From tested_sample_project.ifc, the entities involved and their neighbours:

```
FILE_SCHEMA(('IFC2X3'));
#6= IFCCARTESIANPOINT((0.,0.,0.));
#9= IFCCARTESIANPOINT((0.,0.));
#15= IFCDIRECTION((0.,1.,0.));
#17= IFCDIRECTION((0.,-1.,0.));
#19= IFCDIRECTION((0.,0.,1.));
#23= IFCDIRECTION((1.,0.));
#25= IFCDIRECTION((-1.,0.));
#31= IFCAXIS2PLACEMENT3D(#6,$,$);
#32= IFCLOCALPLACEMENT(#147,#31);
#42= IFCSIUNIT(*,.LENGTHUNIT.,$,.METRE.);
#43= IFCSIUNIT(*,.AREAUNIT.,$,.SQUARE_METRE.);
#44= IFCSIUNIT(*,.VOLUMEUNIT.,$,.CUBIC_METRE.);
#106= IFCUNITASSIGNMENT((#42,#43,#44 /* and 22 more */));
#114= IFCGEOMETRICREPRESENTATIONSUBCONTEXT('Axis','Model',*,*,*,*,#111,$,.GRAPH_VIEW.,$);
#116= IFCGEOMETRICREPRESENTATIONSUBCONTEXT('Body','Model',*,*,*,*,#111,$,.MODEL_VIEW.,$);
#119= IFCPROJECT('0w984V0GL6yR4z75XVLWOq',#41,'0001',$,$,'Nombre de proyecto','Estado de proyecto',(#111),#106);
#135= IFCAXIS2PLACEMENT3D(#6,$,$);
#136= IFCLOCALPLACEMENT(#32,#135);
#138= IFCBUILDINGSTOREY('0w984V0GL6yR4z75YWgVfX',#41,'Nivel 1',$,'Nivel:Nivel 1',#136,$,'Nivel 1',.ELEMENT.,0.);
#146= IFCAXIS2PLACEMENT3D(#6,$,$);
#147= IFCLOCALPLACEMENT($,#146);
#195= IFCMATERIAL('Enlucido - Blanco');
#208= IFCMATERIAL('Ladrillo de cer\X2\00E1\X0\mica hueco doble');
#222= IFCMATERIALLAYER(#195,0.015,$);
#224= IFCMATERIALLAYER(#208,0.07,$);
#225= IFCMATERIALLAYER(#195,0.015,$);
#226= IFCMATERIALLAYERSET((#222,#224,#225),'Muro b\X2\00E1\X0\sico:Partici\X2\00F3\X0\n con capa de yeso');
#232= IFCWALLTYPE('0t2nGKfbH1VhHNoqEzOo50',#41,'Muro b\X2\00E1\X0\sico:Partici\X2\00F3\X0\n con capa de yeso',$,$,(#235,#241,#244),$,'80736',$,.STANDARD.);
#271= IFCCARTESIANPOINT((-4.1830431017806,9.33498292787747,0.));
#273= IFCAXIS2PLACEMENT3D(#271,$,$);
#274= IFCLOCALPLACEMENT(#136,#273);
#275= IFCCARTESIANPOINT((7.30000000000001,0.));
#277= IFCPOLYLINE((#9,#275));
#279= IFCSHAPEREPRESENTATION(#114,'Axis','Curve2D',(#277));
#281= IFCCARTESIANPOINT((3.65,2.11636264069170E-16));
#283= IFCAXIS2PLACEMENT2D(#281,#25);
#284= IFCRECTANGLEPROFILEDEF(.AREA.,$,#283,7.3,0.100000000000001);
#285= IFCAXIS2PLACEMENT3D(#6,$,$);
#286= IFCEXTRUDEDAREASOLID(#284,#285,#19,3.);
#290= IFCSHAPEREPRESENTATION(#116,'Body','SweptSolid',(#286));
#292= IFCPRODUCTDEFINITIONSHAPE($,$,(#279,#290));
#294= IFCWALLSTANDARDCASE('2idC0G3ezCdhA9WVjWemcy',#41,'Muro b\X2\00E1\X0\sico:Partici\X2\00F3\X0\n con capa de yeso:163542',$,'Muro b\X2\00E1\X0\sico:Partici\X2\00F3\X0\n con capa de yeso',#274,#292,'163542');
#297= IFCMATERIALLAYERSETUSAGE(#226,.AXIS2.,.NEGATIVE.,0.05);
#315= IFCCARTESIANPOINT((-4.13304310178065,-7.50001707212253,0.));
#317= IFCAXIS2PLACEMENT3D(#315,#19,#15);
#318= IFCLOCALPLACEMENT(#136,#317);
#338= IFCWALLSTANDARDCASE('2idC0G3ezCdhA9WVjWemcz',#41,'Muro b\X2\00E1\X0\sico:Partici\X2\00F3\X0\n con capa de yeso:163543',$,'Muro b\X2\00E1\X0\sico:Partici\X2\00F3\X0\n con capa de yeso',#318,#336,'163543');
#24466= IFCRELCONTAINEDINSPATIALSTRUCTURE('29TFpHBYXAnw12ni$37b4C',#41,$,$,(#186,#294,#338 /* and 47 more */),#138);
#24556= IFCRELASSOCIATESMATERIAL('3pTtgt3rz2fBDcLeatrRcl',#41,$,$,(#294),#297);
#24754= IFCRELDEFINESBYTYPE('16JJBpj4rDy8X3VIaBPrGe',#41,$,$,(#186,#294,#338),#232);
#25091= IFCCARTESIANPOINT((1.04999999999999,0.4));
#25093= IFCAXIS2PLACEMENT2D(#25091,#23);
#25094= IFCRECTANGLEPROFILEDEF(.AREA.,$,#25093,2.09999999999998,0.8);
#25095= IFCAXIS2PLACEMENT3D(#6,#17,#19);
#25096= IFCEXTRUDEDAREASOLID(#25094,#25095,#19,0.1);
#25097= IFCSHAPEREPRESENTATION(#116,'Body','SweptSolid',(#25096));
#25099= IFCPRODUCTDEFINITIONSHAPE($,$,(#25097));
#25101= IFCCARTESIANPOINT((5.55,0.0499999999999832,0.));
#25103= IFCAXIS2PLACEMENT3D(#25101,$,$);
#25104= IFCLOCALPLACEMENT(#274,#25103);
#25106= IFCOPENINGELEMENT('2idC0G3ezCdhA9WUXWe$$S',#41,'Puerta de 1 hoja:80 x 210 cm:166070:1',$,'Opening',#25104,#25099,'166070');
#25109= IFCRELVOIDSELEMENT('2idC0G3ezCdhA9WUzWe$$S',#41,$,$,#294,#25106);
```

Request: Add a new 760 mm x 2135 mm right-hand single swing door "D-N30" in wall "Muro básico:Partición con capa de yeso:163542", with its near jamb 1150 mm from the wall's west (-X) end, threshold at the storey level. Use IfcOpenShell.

```python
import numpy as np
import ifcopenshell
import ifcopenshell.api.feature
import ifcopenshell.api.geometry
import ifcopenshell.api.root
import ifcopenshell.api.spatial
import ifcopenshell.api.type
import ifcopenshell.geom
import ifcopenshell.util.element
import ifcopenshell.util.placement
import ifcopenshell.util.representation
import ifcopenshell.util.shape
import ifcopenshell.util.unit

model = ifcopenshell.open("tested_sample_project.ifc")
unit_scale = ifcopenshell.util.unit.calculate_unit_scale(model)
settings = ifcopenshell.geom.settings()


def volume(element):
    """Net volume in cubic metres, openings subtracted."""
    shape = ifcopenshell.geom.create_shape(settings, element)
    return ifcopenshell.util.shape.get_volume(shape.geometry)


wall = model.by_id(294)
storey = ifcopenshell.util.element.get_container(wall, ifc_class="IfcBuildingStorey")
context = ifcopenshell.util.representation.get_context(model, "Model", "Body", "MODEL_VIEW")
before = volume(wall)

width, height, from_end, sill = 0.76, 2.135, 1.15, 0.0  # metres

# The wall runs along its own X axis, and the end named is its -X end.
wall_shape = ifcopenshell.geom.create_shape(settings, wall)
x, y, z = ifcopenshell.util.shape.get_vertices(wall_shape.geometry).T
start = x.min() + from_end
face, thickness = float(y.min()), float(y.max() - y.min())
wall_matrix = ifcopenshell.util.placement.get_local_placement(wall.ObjectPlacement)
level = ifcopenshell.util.placement.get_local_placement(storey.ObjectPlacement)[2, 3]


def in_wall(x, y):
    """Placement at x, y metres in the wall's axes, at sill height."""
    matrix = wall_matrix.copy()
    matrix[:, 3] = wall_matrix @ np.array([x / unit_scale, y / unit_scale, 0.0, 1.0])
    matrix[2, 3] = level + sill / unit_scale
    return matrix


# Opening: a box that overshoots both wall faces by 50 mm.
opening = ifcopenshell.api.root.create_entity(model, ifc_class="IfcOpeningElement")
box = ifcopenshell.api.geometry.add_wall_representation(
    model, context=context, length=width, height=height, thickness=thickness + 0.1
)
ifcopenshell.api.geometry.assign_representation(model, product=opening, representation=box)
ifcopenshell.api.geometry.edit_object_placement(model, product=opening, matrix=in_wall(start, face - 0.05), is_si=False)
ifcopenshell.api.feature.add_feature(model, feature=opening, element=wall)

door = ifcopenshell.api.root.create_entity(model, ifc_class="IfcDoor", name="D-N30")
door.OverallWidth, door.OverallHeight = width / unit_scale, height / unit_scale
body = ifcopenshell.api.geometry.add_door_representation(
    model,
    context=context,
    overall_width=door.OverallWidth,
    overall_height=door.OverallHeight,
    operation_type="SINGLE_SWING_RIGHT",
    lining_properties={"LiningDepth": thickness / unit_scale, "ThresholdDepth": thickness / unit_scale},
)
ifcopenshell.api.geometry.assign_representation(model, product=door, representation=body)
ifcopenshell.api.spatial.assign_container(model, products=[door], relating_structure=storey)
fills = ifcopenshell.api.feature.add_filling(model, opening=opening, element=door)
fills.OwnerHistory = door.OwnerHistory  # required in IFC2X3

# IFC2X3 keeps the operation on the door style.
style = ifcopenshell.api.root.create_entity(model, ifc_class="IfcDoorStyle", name="D-N30")
style.OperationType, style.ConstructionType = "SINGLE_SWING_RIGHT", "NOTDEFINED"
style.ParameterTakesPrecedence = style.Sizeable = False
ifcopenshell.api.type.assign_type(model, related_objects=[door], relating_type=style)

# The lining spans the wall, so the door starts at the wall face.
ifcopenshell.api.geometry.edit_object_placement(model, product=door, matrix=in_wall(start, face), is_si=False)

after = volume(wall)

print(f"wall volume {before:.3f} -> {after:.3f} m3")

model.write("tested_sample_project_rev.ifc")
```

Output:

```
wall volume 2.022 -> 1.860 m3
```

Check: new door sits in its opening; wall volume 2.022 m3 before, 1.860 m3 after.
